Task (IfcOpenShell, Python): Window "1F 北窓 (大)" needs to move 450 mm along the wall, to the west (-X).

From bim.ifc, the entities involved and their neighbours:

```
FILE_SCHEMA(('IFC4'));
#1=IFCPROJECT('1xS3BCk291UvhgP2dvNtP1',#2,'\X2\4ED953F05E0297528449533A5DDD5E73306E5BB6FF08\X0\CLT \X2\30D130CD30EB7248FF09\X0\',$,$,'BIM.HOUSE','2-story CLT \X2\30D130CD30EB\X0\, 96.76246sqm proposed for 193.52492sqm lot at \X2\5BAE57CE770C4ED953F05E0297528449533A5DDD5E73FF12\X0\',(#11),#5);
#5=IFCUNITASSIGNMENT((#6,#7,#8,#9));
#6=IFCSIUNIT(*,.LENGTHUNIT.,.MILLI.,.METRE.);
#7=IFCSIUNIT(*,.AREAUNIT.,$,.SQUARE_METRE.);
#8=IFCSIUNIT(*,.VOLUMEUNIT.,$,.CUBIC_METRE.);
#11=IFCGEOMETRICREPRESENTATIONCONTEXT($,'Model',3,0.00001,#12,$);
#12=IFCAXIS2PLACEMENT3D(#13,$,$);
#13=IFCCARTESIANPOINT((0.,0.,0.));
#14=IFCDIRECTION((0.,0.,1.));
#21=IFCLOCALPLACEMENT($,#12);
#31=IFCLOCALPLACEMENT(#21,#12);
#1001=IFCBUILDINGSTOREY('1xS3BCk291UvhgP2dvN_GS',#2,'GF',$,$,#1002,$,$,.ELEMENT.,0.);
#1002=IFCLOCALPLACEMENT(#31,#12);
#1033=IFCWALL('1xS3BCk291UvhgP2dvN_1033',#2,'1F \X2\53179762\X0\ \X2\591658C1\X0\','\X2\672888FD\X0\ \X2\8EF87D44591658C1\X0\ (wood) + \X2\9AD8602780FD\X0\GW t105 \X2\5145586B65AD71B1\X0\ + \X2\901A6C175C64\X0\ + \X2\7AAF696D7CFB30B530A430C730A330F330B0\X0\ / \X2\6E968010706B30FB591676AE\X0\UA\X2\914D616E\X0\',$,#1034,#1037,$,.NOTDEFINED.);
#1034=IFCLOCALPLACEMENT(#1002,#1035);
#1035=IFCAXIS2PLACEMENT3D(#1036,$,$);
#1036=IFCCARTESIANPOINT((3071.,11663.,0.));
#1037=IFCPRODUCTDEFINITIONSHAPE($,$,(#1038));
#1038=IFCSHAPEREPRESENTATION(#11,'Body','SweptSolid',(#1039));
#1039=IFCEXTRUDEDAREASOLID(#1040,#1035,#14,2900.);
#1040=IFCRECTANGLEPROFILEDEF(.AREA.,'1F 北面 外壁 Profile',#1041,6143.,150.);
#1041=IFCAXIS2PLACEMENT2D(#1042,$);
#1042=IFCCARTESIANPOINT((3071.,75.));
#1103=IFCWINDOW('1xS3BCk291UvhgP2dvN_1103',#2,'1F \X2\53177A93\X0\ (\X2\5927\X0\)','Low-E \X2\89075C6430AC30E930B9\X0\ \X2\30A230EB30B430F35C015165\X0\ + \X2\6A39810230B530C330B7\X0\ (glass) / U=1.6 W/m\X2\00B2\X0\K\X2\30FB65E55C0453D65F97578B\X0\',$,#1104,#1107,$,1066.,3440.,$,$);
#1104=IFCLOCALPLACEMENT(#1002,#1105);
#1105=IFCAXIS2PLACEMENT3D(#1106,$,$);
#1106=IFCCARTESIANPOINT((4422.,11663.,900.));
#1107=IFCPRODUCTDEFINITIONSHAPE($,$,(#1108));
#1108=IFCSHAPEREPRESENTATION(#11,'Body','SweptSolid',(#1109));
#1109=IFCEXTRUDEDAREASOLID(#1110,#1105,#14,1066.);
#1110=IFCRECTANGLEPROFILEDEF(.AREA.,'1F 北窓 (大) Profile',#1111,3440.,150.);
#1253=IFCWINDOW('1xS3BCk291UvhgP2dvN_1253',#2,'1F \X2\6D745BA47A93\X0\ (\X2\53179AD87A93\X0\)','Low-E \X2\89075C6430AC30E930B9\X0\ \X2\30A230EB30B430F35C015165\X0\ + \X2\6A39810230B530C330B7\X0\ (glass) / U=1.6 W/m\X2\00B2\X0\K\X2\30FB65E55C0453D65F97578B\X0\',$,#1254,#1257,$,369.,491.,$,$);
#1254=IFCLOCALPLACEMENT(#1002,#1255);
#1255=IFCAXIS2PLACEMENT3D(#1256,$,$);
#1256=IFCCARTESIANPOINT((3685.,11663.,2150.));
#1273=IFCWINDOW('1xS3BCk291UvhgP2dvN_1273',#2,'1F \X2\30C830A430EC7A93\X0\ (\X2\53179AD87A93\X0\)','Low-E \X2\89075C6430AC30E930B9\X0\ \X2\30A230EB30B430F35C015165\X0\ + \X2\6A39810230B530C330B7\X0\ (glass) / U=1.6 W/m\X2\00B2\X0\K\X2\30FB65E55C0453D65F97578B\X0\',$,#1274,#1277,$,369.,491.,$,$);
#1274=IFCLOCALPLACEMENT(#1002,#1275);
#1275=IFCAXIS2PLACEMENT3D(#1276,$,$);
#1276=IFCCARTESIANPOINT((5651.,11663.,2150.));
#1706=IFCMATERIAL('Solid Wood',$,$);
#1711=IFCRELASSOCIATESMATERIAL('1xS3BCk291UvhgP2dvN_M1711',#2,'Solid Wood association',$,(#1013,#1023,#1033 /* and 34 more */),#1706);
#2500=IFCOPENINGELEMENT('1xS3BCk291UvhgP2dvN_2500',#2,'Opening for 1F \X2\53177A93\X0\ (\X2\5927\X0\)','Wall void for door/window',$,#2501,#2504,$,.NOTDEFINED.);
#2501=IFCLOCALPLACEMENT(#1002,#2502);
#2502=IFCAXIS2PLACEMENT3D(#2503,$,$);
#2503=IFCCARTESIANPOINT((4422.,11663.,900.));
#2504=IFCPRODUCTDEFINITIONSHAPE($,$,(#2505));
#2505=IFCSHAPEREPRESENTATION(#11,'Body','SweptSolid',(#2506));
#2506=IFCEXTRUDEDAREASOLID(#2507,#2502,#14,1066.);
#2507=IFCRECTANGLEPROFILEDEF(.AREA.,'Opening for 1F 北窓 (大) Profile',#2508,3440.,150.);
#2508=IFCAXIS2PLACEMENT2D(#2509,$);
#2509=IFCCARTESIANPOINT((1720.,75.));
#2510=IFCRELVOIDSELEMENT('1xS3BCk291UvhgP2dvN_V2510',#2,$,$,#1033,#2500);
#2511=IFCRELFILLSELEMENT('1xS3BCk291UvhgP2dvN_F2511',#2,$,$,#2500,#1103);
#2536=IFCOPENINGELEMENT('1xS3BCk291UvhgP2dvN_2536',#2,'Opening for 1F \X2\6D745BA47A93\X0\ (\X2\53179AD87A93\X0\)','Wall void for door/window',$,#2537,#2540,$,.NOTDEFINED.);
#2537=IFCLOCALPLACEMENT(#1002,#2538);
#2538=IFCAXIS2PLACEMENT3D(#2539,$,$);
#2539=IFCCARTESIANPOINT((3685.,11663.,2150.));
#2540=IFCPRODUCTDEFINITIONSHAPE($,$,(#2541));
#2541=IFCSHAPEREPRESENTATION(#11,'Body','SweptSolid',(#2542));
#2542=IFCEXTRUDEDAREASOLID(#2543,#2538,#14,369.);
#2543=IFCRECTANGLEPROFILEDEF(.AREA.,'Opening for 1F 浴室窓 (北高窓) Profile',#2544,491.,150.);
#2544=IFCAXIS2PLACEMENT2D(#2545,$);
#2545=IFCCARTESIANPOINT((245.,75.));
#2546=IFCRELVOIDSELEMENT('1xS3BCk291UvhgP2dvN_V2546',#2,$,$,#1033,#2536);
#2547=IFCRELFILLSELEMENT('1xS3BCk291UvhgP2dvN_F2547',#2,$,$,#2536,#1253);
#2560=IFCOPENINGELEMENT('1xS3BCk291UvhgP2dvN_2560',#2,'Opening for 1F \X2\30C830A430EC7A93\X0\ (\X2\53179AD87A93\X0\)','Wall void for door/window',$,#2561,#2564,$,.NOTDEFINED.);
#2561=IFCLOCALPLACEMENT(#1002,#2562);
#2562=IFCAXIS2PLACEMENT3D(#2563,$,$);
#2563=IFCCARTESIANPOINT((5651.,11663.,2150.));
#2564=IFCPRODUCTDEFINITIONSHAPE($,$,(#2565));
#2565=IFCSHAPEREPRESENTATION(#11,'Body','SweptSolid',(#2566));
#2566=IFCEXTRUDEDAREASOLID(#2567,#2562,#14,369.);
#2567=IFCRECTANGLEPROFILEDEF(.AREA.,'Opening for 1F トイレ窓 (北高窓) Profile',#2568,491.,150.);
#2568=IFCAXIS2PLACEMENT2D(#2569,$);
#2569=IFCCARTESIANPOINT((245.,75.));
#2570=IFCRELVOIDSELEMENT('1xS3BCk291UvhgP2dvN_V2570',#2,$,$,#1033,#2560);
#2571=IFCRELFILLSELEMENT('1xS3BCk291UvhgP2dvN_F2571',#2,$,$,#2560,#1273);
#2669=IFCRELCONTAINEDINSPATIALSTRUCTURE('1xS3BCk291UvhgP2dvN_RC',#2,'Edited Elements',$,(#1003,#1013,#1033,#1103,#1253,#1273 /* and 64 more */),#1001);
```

```python
import ifcopenshell
import ifcopenshell.api.geometry
import ifcopenshell.util.placement

model = ifcopenshell.open("bim.ifc")

window = model.by_guid("1xS3BCk291UvhgP2dvN_1103")
opening = window.FillsVoids[0].RelatingOpeningElement
wall = opening.VoidsElements[0].RelatingBuildingElement

wall_matrix = ifcopenshell.util.placement.get_local_placement(wall.ObjectPlacement)
shift = wall_matrix[:3, 0] * -450.0
before = ifcopenshell.util.placement.get_local_placement(window.ObjectPlacement)[:3, 3].copy()

# The window is not placed relative to its opening, so move both.
for product in (opening, window):
    matrix = ifcopenshell.util.placement.get_local_placement(product.ObjectPlacement)
    matrix[:3, 3] += shift
    ifcopenshell.api.geometry.edit_object_placement(model, product=product, matrix=matrix, is_si=False)

after = ifcopenshell.util.placement.get_local_placement(window.ObjectPlacement)[:3, 3]
print("window moved by", (after - before).round(3) + 0.0)

model.write("bim_edited.ifc")
```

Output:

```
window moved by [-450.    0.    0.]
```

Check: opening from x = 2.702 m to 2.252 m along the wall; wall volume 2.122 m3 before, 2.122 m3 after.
